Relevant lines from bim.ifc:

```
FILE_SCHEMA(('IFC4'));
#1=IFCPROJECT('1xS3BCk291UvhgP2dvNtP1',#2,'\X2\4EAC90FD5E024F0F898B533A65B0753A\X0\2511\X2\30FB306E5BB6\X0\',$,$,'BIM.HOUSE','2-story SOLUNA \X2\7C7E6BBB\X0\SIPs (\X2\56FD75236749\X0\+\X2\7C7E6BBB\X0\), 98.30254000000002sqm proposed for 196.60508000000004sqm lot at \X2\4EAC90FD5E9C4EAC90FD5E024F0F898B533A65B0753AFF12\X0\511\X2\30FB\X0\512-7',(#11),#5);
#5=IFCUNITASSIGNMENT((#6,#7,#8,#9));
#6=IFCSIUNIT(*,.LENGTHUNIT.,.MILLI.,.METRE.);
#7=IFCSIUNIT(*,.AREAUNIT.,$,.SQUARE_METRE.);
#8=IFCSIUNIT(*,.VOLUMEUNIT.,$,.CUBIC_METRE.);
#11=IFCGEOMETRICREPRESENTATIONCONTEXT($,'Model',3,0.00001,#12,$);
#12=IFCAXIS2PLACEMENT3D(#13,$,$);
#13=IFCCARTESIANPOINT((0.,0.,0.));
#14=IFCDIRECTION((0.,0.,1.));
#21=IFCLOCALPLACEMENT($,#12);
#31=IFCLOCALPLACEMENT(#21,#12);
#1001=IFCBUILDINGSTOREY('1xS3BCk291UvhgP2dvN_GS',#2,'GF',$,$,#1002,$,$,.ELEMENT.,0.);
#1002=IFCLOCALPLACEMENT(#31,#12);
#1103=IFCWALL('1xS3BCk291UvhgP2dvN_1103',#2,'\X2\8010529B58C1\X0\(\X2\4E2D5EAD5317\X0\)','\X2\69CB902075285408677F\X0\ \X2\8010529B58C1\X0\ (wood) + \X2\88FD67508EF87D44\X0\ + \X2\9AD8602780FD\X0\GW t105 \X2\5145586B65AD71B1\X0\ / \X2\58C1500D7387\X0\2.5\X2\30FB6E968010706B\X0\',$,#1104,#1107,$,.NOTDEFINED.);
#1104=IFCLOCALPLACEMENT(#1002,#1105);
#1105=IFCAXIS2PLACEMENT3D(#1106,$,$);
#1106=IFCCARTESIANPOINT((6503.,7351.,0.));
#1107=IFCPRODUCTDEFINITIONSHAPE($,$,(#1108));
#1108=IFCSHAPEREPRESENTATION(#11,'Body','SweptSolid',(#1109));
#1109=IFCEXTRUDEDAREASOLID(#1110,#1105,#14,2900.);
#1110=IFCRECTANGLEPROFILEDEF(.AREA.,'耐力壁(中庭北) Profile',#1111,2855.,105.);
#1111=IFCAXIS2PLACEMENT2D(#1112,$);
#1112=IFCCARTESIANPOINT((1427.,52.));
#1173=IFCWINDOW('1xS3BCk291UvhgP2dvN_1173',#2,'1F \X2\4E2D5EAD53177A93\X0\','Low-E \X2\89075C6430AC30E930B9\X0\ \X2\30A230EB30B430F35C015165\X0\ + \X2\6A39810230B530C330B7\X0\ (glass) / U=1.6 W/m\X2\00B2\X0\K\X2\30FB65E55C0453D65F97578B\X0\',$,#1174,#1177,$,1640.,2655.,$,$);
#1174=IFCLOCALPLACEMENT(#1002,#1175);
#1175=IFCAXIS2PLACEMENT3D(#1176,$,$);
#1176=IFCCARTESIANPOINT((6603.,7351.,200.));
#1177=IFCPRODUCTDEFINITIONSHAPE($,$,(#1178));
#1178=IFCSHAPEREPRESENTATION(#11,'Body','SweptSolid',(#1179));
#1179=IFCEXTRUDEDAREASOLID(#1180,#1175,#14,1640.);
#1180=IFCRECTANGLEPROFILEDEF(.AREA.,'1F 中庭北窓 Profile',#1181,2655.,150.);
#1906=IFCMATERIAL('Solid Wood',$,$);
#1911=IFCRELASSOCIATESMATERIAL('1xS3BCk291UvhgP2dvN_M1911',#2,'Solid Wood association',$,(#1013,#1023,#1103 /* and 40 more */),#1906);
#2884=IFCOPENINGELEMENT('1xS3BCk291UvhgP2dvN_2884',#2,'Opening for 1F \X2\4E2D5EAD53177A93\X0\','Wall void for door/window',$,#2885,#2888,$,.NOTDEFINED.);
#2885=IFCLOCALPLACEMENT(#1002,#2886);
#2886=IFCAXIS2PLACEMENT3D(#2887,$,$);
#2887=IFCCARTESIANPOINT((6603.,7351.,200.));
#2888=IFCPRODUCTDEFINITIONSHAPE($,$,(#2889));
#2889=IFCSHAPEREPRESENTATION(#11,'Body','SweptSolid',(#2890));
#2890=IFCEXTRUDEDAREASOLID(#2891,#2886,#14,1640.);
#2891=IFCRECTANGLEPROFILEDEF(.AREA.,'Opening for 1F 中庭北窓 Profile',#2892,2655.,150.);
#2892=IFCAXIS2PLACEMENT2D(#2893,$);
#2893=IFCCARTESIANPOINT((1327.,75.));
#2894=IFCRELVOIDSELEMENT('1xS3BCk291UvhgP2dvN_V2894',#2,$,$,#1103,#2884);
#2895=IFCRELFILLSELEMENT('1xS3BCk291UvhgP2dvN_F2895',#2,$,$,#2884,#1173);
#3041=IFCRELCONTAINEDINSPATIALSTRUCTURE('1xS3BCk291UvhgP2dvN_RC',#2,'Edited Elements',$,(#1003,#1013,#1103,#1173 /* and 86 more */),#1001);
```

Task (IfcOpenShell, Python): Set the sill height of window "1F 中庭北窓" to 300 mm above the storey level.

```python
import numpy as np
import ifcopenshell
import ifcopenshell.api.geometry
import ifcopenshell.geom
import ifcopenshell.util.element
import ifcopenshell.util.placement
import ifcopenshell.util.shape
import ifcopenshell.util.unit

model = ifcopenshell.open("bim.ifc")
unit_scale = ifcopenshell.util.unit.calculate_unit_scale(model)

window = model.by_guid("1xS3BCk291UvhgP2dvN_1173")
opening = window.FillsVoids[0].RelatingOpeningElement
storey = ifcopenshell.util.element.get_container(window, ifc_class="IfcBuildingStorey")
level = ifcopenshell.util.placement.get_local_placement(storey.ObjectPlacement)[2, 3]

# The opening's origin need not be at the sill, so measure its lowest point.
shape = ifcopenshell.geom.create_shape(ifcopenshell.geom.settings(), opening)
bottom = ifcopenshell.util.shape.get_shape_bottom_elevation(shape, shape.geometry) / unit_scale
dz = level + 0.3 / unit_scale - bottom

shift = np.array([0.0, 0.0, dz])
# The window is not placed relative to its opening, so move both.
for product in (opening, window):
    matrix = ifcopenshell.util.placement.get_local_placement(product.ObjectPlacement)
    matrix[:3, 3] += shift
    ifcopenshell.api.geometry.edit_object_placement(model, product=product, matrix=matrix, is_si=False)

print(f"moved by {dz * unit_scale:+.3f} m")

model.write("bim-out.ifc")
```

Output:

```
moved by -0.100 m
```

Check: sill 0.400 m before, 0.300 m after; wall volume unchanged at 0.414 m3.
